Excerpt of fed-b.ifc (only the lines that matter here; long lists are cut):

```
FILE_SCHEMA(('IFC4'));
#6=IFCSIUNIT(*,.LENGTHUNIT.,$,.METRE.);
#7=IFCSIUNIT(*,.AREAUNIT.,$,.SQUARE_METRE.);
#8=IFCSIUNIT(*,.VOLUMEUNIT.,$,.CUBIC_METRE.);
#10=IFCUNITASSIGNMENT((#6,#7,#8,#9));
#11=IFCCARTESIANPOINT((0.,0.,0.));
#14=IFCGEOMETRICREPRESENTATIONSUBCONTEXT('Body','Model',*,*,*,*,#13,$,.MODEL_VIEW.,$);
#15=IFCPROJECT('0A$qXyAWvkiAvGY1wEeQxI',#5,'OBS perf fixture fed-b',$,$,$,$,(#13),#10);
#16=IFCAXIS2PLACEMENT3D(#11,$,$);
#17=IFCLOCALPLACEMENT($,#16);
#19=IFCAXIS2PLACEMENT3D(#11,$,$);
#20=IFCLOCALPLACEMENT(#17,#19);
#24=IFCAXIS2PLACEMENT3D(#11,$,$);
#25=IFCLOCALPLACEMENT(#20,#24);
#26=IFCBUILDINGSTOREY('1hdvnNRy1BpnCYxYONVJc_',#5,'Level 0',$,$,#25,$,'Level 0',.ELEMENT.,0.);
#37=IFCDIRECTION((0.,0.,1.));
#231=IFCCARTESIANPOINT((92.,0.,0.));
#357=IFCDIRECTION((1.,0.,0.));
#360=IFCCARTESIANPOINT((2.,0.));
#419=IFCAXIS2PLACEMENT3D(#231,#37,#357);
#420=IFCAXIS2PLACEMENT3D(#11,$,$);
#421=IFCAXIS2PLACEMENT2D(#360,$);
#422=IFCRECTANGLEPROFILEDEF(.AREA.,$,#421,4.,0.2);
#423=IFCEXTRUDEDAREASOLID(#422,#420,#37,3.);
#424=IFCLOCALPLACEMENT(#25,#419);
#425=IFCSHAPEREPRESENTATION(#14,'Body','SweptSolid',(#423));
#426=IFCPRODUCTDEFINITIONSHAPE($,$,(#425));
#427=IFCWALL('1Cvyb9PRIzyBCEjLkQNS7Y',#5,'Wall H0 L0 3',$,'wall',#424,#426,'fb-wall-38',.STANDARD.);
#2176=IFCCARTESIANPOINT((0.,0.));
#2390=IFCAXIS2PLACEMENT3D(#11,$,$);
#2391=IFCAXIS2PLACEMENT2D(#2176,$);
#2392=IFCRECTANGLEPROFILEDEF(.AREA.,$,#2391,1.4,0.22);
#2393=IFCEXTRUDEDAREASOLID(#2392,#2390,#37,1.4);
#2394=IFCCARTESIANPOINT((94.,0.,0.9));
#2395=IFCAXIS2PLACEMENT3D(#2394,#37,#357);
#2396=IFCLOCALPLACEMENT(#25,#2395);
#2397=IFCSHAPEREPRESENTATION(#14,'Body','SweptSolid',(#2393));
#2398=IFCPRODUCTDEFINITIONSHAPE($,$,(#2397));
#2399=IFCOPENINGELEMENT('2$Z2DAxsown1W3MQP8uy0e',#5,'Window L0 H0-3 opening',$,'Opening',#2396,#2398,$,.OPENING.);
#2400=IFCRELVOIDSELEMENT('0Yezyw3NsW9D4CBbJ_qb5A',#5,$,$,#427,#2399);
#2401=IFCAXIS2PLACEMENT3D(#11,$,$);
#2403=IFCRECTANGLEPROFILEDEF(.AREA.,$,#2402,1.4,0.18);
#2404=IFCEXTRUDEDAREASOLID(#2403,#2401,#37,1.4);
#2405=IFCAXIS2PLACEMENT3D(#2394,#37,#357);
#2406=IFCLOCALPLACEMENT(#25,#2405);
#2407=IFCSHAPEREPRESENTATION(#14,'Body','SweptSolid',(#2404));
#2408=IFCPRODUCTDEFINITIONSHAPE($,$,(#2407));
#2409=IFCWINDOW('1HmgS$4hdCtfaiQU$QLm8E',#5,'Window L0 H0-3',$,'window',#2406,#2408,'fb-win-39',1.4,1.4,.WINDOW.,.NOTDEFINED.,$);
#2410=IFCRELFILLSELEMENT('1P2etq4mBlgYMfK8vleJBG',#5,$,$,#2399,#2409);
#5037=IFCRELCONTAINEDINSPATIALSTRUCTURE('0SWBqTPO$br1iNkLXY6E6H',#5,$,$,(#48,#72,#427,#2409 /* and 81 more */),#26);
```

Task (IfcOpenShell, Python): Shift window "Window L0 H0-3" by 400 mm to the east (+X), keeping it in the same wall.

```python
import ifcopenshell
import ifcopenshell.api.geometry
import ifcopenshell.util.placement

model = ifcopenshell.open("fed-b.ifc")

window = model.by_guid("1HmgS$4hdCtfaiQU$QLm8E")
opening = window.FillsVoids[0].RelatingOpeningElement
wall = opening.VoidsElements[0].RelatingBuildingElement

wall_matrix = ifcopenshell.util.placement.get_local_placement(wall.ObjectPlacement)
shift = wall_matrix[:3, 0] * 0.4
before = ifcopenshell.util.placement.get_local_placement(window.ObjectPlacement)[:3, 3].copy()

# The window is not placed relative to its opening, so move both.
for product in (opening, window):
    matrix = ifcopenshell.util.placement.get_local_placement(product.ObjectPlacement)
    matrix[:3, 3] += shift
    ifcopenshell.api.geometry.edit_object_placement(model, product=product, matrix=matrix, is_si=False)

after = ifcopenshell.util.placement.get_local_placement(window.ObjectPlacement)[:3, 3]
print("window moved by", (after - before).round(3) + 0.0)

model.write("fed-b_updated.ifc")
```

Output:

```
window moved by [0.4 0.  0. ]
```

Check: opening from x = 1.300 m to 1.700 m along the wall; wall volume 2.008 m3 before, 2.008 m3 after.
